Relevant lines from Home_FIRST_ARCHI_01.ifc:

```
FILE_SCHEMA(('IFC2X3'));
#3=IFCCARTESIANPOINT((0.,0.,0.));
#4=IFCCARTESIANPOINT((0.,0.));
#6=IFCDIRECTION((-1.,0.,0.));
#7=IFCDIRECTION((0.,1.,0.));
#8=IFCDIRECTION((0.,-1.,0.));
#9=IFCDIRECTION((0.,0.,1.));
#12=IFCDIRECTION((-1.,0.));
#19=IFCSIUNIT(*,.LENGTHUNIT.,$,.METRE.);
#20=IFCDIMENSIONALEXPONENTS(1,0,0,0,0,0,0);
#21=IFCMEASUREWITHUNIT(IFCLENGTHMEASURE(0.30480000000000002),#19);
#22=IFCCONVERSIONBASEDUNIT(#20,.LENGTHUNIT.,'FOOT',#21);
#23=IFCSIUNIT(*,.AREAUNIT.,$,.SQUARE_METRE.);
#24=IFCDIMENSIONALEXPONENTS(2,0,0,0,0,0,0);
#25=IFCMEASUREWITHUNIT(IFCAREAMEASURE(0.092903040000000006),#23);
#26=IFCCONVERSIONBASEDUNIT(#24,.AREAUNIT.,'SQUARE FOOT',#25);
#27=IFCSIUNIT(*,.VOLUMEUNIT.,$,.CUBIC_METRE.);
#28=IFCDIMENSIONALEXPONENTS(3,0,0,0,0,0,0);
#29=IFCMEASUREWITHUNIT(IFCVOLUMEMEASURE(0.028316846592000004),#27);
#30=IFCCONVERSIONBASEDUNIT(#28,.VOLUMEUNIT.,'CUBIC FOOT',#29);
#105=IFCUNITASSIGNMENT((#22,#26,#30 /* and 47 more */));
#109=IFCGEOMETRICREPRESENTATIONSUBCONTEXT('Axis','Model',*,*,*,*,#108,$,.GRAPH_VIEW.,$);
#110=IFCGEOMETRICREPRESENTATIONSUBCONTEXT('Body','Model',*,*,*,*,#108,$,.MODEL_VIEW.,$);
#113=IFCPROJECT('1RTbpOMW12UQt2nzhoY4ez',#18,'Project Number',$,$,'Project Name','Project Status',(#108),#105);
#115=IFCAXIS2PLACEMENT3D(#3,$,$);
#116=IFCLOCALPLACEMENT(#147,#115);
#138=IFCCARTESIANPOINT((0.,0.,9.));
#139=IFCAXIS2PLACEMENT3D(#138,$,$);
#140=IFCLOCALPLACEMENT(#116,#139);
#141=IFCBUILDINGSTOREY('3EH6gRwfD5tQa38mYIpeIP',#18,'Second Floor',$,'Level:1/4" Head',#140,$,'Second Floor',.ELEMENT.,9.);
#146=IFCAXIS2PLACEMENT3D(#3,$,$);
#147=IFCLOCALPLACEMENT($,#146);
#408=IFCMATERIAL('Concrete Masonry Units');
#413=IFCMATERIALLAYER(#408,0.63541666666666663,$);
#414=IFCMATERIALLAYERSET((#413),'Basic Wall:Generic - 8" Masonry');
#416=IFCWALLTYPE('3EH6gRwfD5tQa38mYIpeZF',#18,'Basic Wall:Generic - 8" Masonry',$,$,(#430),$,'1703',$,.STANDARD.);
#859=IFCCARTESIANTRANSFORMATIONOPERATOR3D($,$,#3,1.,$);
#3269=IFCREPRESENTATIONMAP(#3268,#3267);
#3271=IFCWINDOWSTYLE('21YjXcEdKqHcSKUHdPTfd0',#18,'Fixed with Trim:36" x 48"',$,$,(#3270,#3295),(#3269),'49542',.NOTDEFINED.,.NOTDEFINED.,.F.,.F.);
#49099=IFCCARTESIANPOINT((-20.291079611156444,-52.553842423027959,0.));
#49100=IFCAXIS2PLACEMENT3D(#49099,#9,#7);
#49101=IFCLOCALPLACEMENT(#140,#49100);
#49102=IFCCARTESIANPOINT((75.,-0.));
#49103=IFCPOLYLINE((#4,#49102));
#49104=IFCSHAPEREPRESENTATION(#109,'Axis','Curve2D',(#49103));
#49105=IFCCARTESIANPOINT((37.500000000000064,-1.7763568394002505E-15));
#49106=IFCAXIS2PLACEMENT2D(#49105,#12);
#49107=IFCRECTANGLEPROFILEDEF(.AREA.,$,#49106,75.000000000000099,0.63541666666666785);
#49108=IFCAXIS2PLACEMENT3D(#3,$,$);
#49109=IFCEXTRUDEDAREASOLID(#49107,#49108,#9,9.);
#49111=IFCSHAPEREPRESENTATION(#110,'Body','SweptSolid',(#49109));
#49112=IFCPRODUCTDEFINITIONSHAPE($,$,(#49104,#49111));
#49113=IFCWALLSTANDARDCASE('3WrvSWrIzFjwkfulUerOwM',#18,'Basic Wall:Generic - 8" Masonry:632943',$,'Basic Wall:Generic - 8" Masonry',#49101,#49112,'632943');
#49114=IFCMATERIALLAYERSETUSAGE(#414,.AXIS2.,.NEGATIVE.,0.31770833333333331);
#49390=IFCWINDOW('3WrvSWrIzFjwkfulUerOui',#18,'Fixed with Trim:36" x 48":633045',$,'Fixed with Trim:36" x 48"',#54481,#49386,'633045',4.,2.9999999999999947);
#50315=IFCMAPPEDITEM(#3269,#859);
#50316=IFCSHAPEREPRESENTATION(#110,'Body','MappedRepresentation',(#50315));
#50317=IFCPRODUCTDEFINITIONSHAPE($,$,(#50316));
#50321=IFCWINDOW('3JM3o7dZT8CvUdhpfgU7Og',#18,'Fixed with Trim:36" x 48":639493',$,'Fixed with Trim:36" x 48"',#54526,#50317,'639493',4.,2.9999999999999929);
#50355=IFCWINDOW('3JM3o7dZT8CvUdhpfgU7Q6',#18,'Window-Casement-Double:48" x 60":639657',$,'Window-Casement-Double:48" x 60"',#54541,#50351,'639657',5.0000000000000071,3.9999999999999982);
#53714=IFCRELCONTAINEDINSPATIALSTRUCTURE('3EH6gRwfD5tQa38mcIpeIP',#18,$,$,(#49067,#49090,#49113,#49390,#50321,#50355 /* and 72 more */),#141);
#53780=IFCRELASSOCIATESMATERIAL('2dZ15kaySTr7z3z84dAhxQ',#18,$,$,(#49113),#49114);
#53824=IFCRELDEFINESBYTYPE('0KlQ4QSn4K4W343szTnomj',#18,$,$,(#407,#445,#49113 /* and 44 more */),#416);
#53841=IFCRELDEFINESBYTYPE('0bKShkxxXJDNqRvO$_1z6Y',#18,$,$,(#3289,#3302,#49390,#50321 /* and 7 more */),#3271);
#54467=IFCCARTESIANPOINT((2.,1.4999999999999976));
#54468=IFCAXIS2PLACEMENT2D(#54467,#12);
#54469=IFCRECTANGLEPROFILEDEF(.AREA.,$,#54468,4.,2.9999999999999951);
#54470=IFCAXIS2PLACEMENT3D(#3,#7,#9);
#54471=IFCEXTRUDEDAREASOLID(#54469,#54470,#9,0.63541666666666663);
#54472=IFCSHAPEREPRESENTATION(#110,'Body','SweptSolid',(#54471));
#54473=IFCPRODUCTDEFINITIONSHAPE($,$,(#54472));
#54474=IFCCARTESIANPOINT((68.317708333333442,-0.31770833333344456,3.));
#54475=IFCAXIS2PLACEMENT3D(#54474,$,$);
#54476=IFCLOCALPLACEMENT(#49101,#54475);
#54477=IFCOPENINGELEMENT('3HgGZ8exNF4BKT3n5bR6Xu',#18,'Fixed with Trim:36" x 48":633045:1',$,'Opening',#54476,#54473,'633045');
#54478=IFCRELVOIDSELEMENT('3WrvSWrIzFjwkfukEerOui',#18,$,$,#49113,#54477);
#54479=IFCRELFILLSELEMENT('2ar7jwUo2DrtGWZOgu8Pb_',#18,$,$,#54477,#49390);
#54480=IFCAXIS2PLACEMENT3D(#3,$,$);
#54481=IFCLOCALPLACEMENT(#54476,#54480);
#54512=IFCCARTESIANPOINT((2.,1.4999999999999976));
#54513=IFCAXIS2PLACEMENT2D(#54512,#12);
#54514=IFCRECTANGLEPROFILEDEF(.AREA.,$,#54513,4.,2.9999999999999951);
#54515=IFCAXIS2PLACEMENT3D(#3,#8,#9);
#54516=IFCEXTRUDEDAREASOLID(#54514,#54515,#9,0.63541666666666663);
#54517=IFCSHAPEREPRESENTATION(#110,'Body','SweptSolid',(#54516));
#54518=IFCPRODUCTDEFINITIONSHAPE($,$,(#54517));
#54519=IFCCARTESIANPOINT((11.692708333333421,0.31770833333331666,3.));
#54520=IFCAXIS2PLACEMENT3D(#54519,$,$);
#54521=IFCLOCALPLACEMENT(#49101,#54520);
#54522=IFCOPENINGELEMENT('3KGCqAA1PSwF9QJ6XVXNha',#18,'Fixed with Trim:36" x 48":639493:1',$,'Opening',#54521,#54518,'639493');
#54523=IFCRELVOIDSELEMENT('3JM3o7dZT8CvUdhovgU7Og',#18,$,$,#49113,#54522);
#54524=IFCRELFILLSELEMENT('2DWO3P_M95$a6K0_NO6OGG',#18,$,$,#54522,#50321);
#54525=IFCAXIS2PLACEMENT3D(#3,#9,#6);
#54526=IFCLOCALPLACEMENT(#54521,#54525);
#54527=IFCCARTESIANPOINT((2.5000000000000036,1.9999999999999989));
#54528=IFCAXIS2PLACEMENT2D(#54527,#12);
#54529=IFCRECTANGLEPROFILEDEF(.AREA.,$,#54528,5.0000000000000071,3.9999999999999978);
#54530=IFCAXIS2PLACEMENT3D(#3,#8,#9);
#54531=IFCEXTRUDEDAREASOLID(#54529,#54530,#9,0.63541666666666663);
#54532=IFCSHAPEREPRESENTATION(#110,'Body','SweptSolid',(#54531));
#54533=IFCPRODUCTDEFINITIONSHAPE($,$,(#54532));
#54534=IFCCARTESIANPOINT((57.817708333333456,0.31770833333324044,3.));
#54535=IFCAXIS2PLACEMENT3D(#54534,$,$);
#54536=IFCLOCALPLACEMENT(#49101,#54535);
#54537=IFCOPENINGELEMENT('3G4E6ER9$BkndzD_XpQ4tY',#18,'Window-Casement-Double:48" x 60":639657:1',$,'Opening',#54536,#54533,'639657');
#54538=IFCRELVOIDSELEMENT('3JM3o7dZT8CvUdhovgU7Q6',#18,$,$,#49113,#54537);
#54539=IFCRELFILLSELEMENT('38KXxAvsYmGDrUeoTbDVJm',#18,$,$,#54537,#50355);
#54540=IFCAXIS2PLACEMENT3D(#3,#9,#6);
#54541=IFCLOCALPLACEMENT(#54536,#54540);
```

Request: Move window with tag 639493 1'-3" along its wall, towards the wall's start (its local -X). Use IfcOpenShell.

```python
import ifcopenshell
import ifcopenshell.api.geometry
import ifcopenshell.util.placement
import ifcopenshell.util.unit

model = ifcopenshell.open("Home_FIRST_ARCHI_01.ifc")
unit_scale = ifcopenshell.util.unit.calculate_unit_scale(model)

window = model.by_id(50321)
opening = window.FillsVoids[0].RelatingOpeningElement
wall = opening.VoidsElements[0].RelatingBuildingElement

wall_matrix = ifcopenshell.util.placement.get_local_placement(wall.ObjectPlacement)
shift = wall_matrix[:3, 0] * -15 * 0.0254 / unit_scale
before = ifcopenshell.util.placement.get_local_placement(window.ObjectPlacement)[:3, 3].copy()

# The window is placed relative to its opening, so it follows when the opening moves.
matrix = ifcopenshell.util.placement.get_local_placement(opening.ObjectPlacement)
matrix[:3, 3] += shift
ifcopenshell.api.geometry.edit_object_placement(
    model, product=opening, matrix=matrix, is_si=False, should_transform_children=True
)

after = ifcopenshell.util.placement.get_local_placement(window.ObjectPlacement)[:3, 3]
print("window moved by", (after - before).round(3) + 0.0)

model.write("Home_FIRST_ARCHI_01-out.ifc")
```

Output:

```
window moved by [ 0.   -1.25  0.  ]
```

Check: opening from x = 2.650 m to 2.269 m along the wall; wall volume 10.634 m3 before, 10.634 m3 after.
